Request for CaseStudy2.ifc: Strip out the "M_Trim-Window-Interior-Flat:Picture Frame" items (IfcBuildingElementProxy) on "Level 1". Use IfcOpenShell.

First a look at what the model holds.

```python
import ifcopenshell
import ifcopenshell.util.element

model = ifcopenshell.open("CaseStudy2.ifc")
print(model.schema)
storey = next(s for s in model.by_type("IfcBuildingStorey") if s.Name == "Level 1")
proxies = [e for e in ifcopenshell.util.element.get_decomposition(storey) if e.is_a("IfcBuildingElementProxy")]
seen = {}
for e in proxies:
    element_type = ifcopenshell.util.element.get_type(e)
    name = element_type.Name if element_type not in (None, e) else None
    seen[name] = seen.get(name, 0) + 1
for name, count in sorted(seen.items(), key=str):
    print(count, "x", name)
```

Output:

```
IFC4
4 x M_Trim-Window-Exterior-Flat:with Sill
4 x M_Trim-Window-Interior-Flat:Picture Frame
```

```python
import ifcopenshell
import ifcopenshell.api.root
import ifcopenshell.util.element

model = ifcopenshell.open("CaseStudy2.ifc")

storey = next(s for s in model.by_type("IfcBuildingStorey") if s.Name == "Level 1")
proxies = [e for e in ifcopenshell.util.element.get_decomposition(storey) if e.is_a("IfcBuildingElementProxy")]
targets = [e for e in proxies if (t := ifcopenshell.util.element.get_type(e)) not in (None, e) and t.Name == "M_Trim-Window-Interior-Flat:Picture Frame"]

for e in targets:
    ifcopenshell.api.root.remove_product(model, product=e)
print(len(targets), "removed")

model.write("CaseStudy2_edited.ifc")
```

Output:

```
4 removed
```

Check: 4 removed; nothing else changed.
